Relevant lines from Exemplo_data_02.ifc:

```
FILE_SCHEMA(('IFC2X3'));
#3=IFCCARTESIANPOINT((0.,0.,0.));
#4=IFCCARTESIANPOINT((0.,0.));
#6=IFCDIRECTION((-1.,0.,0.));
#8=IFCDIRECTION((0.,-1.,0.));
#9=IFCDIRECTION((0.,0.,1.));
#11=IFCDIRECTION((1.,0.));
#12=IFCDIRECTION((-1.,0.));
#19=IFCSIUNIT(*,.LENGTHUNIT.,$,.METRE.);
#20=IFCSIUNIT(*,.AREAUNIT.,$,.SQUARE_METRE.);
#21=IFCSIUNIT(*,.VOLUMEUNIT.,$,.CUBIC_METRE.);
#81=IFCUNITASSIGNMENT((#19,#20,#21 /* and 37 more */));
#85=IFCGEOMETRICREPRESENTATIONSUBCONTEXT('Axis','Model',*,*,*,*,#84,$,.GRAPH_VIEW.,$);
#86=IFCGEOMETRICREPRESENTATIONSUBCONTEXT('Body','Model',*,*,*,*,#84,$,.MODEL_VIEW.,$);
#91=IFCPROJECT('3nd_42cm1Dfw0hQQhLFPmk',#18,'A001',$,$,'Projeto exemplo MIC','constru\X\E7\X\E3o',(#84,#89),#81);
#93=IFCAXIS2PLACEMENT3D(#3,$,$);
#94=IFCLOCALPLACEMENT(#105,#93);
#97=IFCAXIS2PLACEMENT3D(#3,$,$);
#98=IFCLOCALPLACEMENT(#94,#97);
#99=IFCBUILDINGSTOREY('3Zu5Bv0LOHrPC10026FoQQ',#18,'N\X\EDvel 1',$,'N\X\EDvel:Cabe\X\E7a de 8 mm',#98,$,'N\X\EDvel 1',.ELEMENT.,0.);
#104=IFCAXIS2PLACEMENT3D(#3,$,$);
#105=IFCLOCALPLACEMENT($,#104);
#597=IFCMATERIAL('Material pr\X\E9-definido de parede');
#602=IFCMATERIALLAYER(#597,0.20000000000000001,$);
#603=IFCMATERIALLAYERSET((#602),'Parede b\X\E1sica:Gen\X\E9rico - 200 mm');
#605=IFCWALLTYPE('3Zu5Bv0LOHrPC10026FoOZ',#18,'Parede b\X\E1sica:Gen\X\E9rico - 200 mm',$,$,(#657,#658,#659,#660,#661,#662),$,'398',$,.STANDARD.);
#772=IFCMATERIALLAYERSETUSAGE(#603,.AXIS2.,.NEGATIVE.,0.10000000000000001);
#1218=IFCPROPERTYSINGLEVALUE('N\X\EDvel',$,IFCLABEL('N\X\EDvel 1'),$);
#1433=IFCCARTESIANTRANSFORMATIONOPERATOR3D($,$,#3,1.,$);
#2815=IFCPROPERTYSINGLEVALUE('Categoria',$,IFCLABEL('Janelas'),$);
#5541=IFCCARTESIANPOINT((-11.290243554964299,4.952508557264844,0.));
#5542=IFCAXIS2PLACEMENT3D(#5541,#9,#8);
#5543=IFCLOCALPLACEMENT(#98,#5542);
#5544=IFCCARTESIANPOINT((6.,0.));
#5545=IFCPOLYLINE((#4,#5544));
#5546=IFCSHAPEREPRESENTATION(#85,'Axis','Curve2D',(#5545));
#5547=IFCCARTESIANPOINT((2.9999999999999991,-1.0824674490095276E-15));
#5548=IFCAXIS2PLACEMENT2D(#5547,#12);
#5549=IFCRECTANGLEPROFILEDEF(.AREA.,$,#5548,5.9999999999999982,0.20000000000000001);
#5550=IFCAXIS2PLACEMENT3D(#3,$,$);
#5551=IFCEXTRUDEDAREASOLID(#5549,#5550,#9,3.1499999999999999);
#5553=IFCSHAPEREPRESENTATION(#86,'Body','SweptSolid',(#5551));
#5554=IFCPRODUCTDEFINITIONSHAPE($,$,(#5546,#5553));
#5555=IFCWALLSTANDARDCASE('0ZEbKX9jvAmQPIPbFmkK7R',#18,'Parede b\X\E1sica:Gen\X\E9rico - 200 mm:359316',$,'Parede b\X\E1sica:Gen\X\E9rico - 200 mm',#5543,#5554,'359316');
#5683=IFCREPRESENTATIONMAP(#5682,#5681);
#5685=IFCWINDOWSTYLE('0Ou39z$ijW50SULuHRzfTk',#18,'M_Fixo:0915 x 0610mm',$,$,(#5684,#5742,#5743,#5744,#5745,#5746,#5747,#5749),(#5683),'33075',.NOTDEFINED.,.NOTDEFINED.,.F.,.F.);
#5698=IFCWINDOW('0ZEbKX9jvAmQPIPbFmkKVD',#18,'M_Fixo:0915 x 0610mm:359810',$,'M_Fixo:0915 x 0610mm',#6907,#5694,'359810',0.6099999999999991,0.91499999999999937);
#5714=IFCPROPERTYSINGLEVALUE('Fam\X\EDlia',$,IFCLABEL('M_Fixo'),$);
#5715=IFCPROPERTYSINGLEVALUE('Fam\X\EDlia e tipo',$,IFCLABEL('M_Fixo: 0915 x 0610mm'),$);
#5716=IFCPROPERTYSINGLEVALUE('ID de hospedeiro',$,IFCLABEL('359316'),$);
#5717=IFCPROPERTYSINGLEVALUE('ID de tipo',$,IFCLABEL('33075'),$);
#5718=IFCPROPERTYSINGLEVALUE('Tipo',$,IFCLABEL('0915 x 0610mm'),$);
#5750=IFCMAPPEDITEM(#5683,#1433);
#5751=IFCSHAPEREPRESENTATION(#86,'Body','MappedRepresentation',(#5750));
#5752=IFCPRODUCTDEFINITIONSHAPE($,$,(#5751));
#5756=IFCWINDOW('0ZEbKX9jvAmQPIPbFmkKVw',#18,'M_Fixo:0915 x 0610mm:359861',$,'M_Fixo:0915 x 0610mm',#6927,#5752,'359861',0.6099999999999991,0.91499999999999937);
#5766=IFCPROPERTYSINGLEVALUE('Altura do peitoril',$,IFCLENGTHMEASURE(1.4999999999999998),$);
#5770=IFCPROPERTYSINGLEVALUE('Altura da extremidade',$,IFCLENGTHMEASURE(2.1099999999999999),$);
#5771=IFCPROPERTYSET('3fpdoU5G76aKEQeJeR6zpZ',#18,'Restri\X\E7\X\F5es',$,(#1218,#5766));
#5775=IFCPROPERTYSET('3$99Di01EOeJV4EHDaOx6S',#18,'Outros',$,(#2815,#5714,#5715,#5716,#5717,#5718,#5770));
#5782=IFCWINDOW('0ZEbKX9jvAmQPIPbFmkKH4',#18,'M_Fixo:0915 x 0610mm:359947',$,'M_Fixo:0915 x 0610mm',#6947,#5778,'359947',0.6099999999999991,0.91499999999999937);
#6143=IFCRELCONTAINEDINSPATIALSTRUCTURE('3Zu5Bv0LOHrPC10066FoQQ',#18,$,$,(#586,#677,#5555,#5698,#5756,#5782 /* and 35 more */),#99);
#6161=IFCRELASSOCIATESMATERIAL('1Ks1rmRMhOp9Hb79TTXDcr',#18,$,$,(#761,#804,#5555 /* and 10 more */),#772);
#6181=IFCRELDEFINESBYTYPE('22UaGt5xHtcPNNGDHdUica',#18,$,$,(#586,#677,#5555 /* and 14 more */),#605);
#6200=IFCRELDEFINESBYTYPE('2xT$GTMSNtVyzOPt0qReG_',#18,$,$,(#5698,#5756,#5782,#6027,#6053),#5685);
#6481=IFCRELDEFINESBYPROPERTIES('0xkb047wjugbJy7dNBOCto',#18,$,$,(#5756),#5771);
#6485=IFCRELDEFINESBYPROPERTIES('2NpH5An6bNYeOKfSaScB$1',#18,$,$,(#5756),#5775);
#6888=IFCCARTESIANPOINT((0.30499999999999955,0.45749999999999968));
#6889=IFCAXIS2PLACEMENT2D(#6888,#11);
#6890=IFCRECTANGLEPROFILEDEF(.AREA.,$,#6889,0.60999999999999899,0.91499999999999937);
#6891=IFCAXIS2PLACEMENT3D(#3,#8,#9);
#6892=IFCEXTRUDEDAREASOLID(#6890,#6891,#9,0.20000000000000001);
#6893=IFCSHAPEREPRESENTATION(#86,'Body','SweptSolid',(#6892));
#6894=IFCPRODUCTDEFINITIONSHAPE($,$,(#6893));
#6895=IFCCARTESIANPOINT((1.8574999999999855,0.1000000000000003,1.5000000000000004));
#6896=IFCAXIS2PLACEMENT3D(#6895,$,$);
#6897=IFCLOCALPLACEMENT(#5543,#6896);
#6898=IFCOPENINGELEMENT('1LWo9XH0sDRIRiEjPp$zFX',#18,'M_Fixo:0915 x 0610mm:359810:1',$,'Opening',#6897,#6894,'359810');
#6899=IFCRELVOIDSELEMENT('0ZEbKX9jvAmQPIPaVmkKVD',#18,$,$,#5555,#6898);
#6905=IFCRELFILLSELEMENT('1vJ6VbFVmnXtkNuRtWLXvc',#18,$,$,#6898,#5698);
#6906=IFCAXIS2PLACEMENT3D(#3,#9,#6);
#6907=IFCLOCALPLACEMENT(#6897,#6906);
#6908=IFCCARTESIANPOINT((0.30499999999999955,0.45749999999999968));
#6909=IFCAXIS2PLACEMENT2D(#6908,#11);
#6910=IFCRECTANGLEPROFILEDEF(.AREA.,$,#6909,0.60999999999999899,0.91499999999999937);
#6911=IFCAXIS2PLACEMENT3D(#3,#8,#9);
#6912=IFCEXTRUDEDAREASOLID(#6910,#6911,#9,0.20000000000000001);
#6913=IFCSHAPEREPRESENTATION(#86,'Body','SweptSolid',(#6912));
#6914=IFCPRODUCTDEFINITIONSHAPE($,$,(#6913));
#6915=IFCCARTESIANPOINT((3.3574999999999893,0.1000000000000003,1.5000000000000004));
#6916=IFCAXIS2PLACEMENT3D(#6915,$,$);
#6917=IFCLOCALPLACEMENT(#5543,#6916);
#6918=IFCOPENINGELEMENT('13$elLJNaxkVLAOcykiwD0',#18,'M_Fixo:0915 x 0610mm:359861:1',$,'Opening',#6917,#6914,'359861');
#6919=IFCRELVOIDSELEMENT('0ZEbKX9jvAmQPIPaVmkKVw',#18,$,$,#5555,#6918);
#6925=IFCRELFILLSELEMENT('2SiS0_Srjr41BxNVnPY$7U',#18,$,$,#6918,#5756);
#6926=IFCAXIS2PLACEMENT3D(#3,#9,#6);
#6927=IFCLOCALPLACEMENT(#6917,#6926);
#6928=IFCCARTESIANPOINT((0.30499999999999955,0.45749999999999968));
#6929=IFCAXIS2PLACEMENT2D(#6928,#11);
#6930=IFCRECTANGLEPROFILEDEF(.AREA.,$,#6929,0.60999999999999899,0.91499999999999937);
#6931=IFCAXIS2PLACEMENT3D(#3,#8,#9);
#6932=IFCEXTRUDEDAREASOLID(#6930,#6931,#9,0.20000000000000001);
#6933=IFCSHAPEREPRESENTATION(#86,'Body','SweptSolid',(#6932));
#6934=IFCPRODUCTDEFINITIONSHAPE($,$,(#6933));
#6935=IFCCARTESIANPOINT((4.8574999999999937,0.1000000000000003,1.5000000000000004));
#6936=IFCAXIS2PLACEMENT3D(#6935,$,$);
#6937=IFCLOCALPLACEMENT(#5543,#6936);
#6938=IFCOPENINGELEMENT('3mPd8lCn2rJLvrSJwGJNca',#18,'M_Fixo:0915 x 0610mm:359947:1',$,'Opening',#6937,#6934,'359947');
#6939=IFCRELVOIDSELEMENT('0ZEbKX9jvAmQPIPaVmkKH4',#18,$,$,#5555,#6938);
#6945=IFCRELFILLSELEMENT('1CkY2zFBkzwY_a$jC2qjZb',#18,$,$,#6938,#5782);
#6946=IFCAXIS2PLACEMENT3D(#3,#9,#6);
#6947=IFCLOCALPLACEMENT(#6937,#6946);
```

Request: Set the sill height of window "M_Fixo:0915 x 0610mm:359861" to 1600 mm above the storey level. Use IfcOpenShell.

```python
import numpy as np
import ifcopenshell
import ifcopenshell.api.geometry
import ifcopenshell.api.pset
import ifcopenshell.geom
import ifcopenshell.util.element
import ifcopenshell.util.placement
import ifcopenshell.util.shape
import ifcopenshell.util.unit

model = ifcopenshell.open("Exemplo_data_02.ifc")
unit_scale = ifcopenshell.util.unit.calculate_unit_scale(model)

window = model.by_guid("0ZEbKX9jvAmQPIPbFmkKVw")
opening = window.FillsVoids[0].RelatingOpeningElement
storey = ifcopenshell.util.element.get_container(window, ifc_class="IfcBuildingStorey")
level = ifcopenshell.util.placement.get_local_placement(storey.ObjectPlacement)[2, 3]

# The opening's origin need not be at the sill, so measure its lowest point.
shape = ifcopenshell.geom.create_shape(ifcopenshell.geom.settings(), opening)
bottom = ifcopenshell.util.shape.get_shape_bottom_elevation(shape, shape.geometry) / unit_scale
dz = level + 1.6 / unit_scale - bottom

shift = np.array([0.0, 0.0, dz])
# The window is placed relative to its opening, so it follows when the opening moves.
matrix = ifcopenshell.util.placement.get_local_placement(opening.ObjectPlacement)
matrix[:3, 3] += shift
ifcopenshell.api.geometry.edit_object_placement(
    model, product=opening, matrix=matrix, is_si=False, should_transform_children=True
)

# Keep the stored heights in step.
pset = model.by_id(ifcopenshell.util.element.get_pset(window, "Restrições", should_inherit=False)["id"])
ifcopenshell.api.pset.edit_pset(model, pset=pset, properties={
    "Altura do peitoril": model.create_entity("IfcLengthMeasure", ifcopenshell.util.element.get_pset(window, "Restrições", "Altura do peitoril") + dz),
})
pset = model.by_id(ifcopenshell.util.element.get_pset(window, "Outros", should_inherit=False)["id"])
ifcopenshell.api.pset.edit_pset(model, pset=pset, properties={
    "Altura da extremidade": model.create_entity("IfcLengthMeasure", ifcopenshell.util.element.get_pset(window, "Outros", "Altura da extremidade") + dz),
})

print(f"moved by {dz * unit_scale:+.3f} m")

model.write("Exemplo_data_02_updated.ifc")
```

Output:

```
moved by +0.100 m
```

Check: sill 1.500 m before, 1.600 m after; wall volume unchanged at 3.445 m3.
